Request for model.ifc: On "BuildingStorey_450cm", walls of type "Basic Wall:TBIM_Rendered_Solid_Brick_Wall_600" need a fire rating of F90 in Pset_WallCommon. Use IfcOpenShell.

First a look at what the model holds.

```python
import ifcopenshell
import ifcopenshell.util.element

model = ifcopenshell.open("model.ifc")
print(model.schema)
storey = next(s for s in model.by_type("IfcBuildingStorey") if s.Name == "BuildingStorey_450cm")
walls = [e for e in ifcopenshell.util.element.get_decomposition(storey) if e.is_a("IfcWall")]
seen = {}
for e in walls:
    element_type = ifcopenshell.util.element.get_type(e)
    key = (element_type.Name if element_type != e and element_type else None, ifcopenshell.util.element.get_pset(e, "Pset_WallCommon", "FireRating"))
    seen[key] = seen.get(key, 0) + 1
for (name, value), count in sorted(seen.items(), key=str):
    print(count, "x", name, "|", value)
```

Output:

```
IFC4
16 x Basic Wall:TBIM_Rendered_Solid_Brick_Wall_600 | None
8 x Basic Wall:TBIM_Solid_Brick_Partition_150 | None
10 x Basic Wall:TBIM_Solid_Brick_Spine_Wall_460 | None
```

```python
import ifcopenshell
import ifcopenshell.api.pset
import ifcopenshell.util.element

model = ifcopenshell.open("model.ifc")

storey = next(s for s in model.by_type("IfcBuildingStorey") if s.Name == "BuildingStorey_450cm")
walls = [e for e in ifcopenshell.util.element.get_decomposition(storey) if e.is_a("IfcWall")]

count = 0
for e in walls:
    element_type = ifcopenshell.util.element.get_type(e)
    if element_type in (None, e) or element_type.Name != "Basic Wall:TBIM_Rendered_Solid_Brick_Wall_600":
        continue
    # add_pset returns the element's existing set when there is one.
    pset = ifcopenshell.api.pset.add_pset(model, product=e, name="Pset_WallCommon")
    ifcopenshell.api.pset.edit_pset(model, pset=pset, properties={"FireRating": "F90"})
    count += 1

print(count, "walls updated")

model.write("model_edited.ifc")
```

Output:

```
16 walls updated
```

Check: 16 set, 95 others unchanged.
